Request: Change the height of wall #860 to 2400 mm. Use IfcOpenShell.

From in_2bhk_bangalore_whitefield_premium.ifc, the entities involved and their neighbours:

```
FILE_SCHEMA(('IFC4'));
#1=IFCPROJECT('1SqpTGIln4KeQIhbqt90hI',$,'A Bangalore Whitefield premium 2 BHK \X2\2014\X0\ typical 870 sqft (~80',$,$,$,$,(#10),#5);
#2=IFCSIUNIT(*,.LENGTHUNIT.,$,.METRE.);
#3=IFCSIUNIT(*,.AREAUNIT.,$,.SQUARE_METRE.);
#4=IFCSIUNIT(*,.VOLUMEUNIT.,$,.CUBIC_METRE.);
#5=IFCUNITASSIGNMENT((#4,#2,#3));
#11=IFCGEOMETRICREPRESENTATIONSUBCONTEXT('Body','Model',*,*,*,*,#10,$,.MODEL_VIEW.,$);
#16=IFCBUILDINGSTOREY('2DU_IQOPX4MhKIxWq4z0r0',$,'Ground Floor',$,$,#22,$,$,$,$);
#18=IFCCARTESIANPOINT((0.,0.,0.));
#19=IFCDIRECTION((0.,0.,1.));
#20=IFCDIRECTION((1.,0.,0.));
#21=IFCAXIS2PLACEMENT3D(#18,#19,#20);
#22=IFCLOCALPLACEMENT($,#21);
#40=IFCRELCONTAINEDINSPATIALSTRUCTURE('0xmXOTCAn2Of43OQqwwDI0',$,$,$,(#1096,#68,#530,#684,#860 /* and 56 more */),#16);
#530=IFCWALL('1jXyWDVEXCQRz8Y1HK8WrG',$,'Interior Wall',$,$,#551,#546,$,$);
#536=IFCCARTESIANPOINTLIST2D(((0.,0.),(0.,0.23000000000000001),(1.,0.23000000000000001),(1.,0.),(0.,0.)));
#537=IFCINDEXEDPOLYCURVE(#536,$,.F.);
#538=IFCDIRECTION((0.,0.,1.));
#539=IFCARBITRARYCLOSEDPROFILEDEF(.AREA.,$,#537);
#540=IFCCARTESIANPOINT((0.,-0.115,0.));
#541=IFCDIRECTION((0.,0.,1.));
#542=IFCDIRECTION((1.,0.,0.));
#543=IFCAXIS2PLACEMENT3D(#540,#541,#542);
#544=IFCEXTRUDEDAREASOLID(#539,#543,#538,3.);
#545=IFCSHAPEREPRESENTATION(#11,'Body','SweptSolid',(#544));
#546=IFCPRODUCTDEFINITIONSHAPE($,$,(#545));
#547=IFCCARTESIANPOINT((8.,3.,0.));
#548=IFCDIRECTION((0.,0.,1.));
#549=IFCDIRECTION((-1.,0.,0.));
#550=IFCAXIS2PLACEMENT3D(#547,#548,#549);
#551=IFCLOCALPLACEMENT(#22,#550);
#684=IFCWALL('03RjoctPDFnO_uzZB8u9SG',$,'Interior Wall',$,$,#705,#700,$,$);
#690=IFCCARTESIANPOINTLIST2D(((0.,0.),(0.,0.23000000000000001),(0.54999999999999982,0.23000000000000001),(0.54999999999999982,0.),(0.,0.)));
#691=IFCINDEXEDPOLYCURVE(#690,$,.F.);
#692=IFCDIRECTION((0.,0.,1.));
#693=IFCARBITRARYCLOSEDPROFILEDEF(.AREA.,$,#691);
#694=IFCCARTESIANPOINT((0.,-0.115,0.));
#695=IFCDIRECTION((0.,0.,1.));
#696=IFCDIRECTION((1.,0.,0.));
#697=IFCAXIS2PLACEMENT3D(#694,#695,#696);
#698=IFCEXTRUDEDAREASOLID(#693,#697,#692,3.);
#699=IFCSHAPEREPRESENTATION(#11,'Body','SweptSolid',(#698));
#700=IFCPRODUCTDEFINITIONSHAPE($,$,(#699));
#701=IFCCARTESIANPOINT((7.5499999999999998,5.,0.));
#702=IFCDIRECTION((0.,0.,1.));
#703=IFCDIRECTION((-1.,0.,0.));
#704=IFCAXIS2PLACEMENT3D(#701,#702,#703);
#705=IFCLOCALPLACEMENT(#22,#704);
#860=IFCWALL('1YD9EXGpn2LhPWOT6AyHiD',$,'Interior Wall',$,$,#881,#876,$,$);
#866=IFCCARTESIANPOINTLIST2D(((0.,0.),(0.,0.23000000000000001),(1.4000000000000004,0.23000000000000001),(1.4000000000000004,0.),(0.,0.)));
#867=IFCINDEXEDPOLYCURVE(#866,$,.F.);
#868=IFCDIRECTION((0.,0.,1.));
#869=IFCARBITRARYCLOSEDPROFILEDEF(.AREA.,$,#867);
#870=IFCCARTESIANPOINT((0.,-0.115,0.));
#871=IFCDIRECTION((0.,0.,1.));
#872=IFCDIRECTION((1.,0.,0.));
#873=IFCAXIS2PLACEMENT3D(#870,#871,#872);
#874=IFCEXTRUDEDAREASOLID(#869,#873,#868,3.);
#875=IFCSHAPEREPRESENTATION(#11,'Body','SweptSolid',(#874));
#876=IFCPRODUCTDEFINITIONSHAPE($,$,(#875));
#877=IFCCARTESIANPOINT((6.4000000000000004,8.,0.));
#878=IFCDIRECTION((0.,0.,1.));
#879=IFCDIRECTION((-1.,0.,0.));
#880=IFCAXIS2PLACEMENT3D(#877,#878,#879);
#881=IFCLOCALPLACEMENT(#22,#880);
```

```python
import ifcopenshell
import ifcopenshell.geom
import ifcopenshell.util.representation
import ifcopenshell.util.shape

model = ifcopenshell.open("in_2bhk_bangalore_whitefield_premium.ifc")
settings = ifcopenshell.geom.settings()


def volume(element):
    """Net volume in cubic metres, openings subtracted."""
    shape = ifcopenshell.geom.create_shape(settings, element)
    return ifcopenshell.util.shape.get_volume(shape.geometry)


wall = model.by_guid("1YD9EXGpn2LhPWOT6AyHiD")
before = volume(wall)

body = ifcopenshell.util.representation.get_representation(wall, "Model", "Body")
solid = body.Items[0]
old_height = solid.Depth
solid.Depth = 2.4
after = volume(wall)

print(f"height {old_height:g} -> {solid.Depth:g}, volume {before:.3f} -> {after:.3f} m3")

model.write("in_2bhk_bangalore_whitefield_premium_v2.ifc")
```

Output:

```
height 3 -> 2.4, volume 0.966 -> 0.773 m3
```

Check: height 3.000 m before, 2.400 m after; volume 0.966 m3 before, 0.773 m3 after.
